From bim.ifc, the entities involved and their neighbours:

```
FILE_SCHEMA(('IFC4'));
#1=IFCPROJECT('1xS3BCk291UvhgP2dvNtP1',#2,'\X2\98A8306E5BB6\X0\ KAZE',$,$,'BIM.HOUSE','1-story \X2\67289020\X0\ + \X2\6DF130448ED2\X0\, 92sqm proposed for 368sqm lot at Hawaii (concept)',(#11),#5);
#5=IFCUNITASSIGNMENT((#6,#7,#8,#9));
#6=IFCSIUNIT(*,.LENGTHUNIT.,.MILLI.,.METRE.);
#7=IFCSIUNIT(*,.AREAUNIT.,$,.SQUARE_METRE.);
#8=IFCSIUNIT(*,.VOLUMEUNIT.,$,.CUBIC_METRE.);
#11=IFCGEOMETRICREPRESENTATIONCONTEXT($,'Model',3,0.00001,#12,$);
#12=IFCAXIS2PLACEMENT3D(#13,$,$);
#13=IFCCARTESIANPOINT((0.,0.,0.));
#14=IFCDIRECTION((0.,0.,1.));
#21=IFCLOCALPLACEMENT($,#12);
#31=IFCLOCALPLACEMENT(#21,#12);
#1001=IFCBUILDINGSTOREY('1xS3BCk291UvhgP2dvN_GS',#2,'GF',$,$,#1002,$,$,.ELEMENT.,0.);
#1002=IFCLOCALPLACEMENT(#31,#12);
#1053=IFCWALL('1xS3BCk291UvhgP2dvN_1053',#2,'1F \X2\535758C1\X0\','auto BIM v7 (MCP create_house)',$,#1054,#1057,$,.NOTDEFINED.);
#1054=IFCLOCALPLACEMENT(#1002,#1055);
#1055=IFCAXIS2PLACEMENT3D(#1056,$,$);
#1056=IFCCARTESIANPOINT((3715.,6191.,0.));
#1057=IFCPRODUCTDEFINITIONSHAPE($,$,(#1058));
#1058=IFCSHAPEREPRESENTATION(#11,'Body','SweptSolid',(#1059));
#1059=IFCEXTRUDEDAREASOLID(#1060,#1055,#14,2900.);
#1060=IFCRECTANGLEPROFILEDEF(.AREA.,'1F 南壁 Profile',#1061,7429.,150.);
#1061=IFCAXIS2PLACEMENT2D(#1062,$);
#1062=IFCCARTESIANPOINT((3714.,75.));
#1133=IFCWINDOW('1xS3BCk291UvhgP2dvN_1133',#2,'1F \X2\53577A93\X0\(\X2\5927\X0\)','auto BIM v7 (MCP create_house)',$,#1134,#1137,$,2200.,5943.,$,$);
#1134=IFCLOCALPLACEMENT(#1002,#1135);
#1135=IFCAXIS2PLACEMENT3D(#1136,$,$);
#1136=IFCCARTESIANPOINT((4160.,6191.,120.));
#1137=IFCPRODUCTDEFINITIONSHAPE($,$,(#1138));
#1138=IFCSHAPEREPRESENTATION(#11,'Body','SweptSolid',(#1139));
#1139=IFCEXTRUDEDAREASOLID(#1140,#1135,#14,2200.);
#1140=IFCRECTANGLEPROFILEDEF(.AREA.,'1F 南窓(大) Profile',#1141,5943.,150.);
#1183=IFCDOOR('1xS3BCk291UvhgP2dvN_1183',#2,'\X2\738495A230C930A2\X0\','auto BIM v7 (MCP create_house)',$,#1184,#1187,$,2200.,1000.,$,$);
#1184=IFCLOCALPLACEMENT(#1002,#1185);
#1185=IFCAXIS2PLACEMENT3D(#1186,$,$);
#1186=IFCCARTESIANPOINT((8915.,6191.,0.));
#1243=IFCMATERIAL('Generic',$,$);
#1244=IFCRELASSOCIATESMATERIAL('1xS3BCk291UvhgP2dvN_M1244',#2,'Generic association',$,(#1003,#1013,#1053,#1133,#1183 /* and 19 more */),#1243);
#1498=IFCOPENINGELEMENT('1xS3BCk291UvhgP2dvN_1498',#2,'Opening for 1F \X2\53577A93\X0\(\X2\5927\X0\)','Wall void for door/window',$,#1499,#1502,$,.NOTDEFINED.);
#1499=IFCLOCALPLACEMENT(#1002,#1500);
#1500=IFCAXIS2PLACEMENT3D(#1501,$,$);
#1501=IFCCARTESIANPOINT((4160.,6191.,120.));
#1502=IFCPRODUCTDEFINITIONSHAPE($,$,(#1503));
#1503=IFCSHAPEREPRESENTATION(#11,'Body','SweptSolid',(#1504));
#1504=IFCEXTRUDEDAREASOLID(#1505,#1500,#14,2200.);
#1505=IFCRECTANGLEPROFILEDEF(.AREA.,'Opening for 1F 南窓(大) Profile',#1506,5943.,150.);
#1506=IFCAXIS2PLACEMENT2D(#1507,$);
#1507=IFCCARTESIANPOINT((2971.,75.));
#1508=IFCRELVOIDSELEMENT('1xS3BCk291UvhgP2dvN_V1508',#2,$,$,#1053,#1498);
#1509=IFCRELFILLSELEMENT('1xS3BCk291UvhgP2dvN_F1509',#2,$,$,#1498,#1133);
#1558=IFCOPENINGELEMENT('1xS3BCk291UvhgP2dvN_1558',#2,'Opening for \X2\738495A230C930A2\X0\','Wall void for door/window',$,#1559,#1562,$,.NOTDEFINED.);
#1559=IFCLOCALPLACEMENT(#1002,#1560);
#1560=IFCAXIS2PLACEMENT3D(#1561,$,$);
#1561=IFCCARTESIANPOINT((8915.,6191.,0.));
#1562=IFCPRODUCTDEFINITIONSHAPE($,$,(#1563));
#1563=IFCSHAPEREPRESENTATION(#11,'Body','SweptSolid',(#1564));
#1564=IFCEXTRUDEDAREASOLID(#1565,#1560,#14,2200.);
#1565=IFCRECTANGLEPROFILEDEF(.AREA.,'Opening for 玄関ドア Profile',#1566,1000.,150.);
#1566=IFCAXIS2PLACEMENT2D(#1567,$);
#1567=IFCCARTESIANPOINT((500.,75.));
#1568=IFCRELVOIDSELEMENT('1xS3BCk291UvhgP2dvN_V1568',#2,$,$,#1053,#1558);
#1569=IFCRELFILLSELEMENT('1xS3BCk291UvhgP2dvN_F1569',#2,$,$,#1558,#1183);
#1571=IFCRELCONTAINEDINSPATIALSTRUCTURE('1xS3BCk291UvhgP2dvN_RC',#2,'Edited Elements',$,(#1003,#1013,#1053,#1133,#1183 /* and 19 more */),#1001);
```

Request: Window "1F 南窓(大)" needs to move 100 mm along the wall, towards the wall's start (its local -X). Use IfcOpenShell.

```python
import ifcopenshell
import ifcopenshell.api.geometry
import ifcopenshell.util.placement

model = ifcopenshell.open("bim.ifc")

window = model.by_guid("1xS3BCk291UvhgP2dvN_1133")
opening = window.FillsVoids[0].RelatingOpeningElement
wall = opening.VoidsElements[0].RelatingBuildingElement

wall_matrix = ifcopenshell.util.placement.get_local_placement(wall.ObjectPlacement)
shift = wall_matrix[:3, 0] * -100.0
before = ifcopenshell.util.placement.get_local_placement(window.ObjectPlacement)[:3, 3].copy()

# The window is not placed relative to its opening, so move both.
for product in (opening, window):
    matrix = ifcopenshell.util.placement.get_local_placement(product.ObjectPlacement)
    matrix[:3, 3] += shift
    ifcopenshell.api.geometry.edit_object_placement(model, product=product, matrix=matrix, is_si=False)

after = ifcopenshell.util.placement.get_local_placement(window.ObjectPlacement)[:3, 3]
print("window moved by", (after - before).round(3) + 0.0)

model.write("bim_edited.ifc")
```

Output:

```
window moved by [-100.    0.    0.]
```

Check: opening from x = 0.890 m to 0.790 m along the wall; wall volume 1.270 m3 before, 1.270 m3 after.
